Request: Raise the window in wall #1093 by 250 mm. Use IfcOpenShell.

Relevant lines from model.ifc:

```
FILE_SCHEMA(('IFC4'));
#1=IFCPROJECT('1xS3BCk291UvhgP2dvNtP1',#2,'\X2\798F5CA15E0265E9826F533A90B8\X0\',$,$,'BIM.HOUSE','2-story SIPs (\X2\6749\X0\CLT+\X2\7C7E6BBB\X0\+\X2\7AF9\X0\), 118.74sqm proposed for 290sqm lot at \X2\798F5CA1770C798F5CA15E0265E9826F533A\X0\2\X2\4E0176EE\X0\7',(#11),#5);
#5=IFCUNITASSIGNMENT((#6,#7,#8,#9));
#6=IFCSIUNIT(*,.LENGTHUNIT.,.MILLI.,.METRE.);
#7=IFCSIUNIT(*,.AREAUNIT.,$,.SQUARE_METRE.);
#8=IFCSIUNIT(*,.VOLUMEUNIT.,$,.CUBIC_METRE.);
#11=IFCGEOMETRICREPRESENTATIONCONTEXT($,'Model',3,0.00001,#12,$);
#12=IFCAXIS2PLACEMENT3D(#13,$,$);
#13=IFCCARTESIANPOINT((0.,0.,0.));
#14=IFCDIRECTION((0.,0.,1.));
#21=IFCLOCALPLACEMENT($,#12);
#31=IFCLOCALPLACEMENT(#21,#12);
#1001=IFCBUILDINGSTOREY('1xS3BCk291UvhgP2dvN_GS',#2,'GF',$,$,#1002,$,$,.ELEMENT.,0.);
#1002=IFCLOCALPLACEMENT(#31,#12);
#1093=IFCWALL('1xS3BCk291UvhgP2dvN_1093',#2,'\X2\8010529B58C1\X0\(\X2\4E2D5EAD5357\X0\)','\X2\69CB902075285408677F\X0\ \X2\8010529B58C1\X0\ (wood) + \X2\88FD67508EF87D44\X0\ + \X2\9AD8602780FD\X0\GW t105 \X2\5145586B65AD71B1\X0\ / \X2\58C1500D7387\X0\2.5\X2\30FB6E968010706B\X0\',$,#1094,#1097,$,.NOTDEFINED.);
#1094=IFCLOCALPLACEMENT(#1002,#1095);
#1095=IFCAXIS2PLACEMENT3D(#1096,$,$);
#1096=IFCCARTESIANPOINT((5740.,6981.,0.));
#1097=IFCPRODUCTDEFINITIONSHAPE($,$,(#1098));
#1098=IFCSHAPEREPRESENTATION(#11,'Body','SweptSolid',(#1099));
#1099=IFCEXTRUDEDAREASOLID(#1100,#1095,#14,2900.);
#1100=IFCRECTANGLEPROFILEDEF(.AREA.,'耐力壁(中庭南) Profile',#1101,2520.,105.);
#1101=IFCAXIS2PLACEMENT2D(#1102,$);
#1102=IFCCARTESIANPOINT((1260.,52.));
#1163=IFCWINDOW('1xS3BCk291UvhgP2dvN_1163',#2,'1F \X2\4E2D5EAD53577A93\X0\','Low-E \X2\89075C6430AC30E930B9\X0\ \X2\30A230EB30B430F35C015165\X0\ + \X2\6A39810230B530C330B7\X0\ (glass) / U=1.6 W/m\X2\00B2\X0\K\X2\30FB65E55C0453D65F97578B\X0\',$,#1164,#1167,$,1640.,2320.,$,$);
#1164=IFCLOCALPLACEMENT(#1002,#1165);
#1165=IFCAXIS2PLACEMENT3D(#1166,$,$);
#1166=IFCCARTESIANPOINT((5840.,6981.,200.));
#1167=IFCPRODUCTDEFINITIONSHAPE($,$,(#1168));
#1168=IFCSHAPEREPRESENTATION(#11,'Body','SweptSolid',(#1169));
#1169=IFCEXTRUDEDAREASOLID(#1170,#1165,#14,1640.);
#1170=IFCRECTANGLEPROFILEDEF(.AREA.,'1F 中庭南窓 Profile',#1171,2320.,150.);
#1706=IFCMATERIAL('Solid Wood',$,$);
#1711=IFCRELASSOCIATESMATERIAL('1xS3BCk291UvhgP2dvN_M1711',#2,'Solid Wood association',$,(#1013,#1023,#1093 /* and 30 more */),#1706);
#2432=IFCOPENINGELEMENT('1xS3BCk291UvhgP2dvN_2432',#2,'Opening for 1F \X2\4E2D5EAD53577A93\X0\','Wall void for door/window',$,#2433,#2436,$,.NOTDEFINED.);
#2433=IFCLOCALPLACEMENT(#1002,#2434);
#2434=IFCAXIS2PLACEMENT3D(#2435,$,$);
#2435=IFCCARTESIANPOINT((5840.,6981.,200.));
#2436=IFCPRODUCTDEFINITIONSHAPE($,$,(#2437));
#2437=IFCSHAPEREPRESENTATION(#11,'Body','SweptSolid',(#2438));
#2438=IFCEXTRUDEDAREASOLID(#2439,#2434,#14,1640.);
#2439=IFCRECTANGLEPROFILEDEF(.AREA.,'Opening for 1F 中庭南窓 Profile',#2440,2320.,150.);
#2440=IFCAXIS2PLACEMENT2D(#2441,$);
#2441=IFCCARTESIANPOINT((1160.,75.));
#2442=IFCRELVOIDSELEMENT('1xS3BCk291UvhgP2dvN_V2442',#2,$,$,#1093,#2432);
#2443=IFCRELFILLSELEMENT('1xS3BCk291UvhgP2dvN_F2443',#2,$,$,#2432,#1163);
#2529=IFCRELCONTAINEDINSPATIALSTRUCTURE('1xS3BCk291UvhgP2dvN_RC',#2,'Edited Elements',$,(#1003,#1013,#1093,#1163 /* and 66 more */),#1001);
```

```python
import numpy as np
import ifcopenshell
import ifcopenshell.api.geometry
import ifcopenshell.util.placement
import ifcopenshell.util.unit

model = ifcopenshell.open("model.ifc")
unit_scale = ifcopenshell.util.unit.calculate_unit_scale(model)

window = model.by_guid("1xS3BCk291UvhgP2dvN_1163")
opening = window.FillsVoids[0].RelatingOpeningElement
dz = 250.0

shift = np.array([0.0, 0.0, dz])
# The window is not placed relative to its opening, so move both.
for product in (opening, window):
    matrix = ifcopenshell.util.placement.get_local_placement(product.ObjectPlacement)
    matrix[:3, 3] += shift
    ifcopenshell.api.geometry.edit_object_placement(model, product=product, matrix=matrix, is_si=False)

print(f"moved by {dz * unit_scale:+.3f} m")

model.write("model_edited.ifc")
```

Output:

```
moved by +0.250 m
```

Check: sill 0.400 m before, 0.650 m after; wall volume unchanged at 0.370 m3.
